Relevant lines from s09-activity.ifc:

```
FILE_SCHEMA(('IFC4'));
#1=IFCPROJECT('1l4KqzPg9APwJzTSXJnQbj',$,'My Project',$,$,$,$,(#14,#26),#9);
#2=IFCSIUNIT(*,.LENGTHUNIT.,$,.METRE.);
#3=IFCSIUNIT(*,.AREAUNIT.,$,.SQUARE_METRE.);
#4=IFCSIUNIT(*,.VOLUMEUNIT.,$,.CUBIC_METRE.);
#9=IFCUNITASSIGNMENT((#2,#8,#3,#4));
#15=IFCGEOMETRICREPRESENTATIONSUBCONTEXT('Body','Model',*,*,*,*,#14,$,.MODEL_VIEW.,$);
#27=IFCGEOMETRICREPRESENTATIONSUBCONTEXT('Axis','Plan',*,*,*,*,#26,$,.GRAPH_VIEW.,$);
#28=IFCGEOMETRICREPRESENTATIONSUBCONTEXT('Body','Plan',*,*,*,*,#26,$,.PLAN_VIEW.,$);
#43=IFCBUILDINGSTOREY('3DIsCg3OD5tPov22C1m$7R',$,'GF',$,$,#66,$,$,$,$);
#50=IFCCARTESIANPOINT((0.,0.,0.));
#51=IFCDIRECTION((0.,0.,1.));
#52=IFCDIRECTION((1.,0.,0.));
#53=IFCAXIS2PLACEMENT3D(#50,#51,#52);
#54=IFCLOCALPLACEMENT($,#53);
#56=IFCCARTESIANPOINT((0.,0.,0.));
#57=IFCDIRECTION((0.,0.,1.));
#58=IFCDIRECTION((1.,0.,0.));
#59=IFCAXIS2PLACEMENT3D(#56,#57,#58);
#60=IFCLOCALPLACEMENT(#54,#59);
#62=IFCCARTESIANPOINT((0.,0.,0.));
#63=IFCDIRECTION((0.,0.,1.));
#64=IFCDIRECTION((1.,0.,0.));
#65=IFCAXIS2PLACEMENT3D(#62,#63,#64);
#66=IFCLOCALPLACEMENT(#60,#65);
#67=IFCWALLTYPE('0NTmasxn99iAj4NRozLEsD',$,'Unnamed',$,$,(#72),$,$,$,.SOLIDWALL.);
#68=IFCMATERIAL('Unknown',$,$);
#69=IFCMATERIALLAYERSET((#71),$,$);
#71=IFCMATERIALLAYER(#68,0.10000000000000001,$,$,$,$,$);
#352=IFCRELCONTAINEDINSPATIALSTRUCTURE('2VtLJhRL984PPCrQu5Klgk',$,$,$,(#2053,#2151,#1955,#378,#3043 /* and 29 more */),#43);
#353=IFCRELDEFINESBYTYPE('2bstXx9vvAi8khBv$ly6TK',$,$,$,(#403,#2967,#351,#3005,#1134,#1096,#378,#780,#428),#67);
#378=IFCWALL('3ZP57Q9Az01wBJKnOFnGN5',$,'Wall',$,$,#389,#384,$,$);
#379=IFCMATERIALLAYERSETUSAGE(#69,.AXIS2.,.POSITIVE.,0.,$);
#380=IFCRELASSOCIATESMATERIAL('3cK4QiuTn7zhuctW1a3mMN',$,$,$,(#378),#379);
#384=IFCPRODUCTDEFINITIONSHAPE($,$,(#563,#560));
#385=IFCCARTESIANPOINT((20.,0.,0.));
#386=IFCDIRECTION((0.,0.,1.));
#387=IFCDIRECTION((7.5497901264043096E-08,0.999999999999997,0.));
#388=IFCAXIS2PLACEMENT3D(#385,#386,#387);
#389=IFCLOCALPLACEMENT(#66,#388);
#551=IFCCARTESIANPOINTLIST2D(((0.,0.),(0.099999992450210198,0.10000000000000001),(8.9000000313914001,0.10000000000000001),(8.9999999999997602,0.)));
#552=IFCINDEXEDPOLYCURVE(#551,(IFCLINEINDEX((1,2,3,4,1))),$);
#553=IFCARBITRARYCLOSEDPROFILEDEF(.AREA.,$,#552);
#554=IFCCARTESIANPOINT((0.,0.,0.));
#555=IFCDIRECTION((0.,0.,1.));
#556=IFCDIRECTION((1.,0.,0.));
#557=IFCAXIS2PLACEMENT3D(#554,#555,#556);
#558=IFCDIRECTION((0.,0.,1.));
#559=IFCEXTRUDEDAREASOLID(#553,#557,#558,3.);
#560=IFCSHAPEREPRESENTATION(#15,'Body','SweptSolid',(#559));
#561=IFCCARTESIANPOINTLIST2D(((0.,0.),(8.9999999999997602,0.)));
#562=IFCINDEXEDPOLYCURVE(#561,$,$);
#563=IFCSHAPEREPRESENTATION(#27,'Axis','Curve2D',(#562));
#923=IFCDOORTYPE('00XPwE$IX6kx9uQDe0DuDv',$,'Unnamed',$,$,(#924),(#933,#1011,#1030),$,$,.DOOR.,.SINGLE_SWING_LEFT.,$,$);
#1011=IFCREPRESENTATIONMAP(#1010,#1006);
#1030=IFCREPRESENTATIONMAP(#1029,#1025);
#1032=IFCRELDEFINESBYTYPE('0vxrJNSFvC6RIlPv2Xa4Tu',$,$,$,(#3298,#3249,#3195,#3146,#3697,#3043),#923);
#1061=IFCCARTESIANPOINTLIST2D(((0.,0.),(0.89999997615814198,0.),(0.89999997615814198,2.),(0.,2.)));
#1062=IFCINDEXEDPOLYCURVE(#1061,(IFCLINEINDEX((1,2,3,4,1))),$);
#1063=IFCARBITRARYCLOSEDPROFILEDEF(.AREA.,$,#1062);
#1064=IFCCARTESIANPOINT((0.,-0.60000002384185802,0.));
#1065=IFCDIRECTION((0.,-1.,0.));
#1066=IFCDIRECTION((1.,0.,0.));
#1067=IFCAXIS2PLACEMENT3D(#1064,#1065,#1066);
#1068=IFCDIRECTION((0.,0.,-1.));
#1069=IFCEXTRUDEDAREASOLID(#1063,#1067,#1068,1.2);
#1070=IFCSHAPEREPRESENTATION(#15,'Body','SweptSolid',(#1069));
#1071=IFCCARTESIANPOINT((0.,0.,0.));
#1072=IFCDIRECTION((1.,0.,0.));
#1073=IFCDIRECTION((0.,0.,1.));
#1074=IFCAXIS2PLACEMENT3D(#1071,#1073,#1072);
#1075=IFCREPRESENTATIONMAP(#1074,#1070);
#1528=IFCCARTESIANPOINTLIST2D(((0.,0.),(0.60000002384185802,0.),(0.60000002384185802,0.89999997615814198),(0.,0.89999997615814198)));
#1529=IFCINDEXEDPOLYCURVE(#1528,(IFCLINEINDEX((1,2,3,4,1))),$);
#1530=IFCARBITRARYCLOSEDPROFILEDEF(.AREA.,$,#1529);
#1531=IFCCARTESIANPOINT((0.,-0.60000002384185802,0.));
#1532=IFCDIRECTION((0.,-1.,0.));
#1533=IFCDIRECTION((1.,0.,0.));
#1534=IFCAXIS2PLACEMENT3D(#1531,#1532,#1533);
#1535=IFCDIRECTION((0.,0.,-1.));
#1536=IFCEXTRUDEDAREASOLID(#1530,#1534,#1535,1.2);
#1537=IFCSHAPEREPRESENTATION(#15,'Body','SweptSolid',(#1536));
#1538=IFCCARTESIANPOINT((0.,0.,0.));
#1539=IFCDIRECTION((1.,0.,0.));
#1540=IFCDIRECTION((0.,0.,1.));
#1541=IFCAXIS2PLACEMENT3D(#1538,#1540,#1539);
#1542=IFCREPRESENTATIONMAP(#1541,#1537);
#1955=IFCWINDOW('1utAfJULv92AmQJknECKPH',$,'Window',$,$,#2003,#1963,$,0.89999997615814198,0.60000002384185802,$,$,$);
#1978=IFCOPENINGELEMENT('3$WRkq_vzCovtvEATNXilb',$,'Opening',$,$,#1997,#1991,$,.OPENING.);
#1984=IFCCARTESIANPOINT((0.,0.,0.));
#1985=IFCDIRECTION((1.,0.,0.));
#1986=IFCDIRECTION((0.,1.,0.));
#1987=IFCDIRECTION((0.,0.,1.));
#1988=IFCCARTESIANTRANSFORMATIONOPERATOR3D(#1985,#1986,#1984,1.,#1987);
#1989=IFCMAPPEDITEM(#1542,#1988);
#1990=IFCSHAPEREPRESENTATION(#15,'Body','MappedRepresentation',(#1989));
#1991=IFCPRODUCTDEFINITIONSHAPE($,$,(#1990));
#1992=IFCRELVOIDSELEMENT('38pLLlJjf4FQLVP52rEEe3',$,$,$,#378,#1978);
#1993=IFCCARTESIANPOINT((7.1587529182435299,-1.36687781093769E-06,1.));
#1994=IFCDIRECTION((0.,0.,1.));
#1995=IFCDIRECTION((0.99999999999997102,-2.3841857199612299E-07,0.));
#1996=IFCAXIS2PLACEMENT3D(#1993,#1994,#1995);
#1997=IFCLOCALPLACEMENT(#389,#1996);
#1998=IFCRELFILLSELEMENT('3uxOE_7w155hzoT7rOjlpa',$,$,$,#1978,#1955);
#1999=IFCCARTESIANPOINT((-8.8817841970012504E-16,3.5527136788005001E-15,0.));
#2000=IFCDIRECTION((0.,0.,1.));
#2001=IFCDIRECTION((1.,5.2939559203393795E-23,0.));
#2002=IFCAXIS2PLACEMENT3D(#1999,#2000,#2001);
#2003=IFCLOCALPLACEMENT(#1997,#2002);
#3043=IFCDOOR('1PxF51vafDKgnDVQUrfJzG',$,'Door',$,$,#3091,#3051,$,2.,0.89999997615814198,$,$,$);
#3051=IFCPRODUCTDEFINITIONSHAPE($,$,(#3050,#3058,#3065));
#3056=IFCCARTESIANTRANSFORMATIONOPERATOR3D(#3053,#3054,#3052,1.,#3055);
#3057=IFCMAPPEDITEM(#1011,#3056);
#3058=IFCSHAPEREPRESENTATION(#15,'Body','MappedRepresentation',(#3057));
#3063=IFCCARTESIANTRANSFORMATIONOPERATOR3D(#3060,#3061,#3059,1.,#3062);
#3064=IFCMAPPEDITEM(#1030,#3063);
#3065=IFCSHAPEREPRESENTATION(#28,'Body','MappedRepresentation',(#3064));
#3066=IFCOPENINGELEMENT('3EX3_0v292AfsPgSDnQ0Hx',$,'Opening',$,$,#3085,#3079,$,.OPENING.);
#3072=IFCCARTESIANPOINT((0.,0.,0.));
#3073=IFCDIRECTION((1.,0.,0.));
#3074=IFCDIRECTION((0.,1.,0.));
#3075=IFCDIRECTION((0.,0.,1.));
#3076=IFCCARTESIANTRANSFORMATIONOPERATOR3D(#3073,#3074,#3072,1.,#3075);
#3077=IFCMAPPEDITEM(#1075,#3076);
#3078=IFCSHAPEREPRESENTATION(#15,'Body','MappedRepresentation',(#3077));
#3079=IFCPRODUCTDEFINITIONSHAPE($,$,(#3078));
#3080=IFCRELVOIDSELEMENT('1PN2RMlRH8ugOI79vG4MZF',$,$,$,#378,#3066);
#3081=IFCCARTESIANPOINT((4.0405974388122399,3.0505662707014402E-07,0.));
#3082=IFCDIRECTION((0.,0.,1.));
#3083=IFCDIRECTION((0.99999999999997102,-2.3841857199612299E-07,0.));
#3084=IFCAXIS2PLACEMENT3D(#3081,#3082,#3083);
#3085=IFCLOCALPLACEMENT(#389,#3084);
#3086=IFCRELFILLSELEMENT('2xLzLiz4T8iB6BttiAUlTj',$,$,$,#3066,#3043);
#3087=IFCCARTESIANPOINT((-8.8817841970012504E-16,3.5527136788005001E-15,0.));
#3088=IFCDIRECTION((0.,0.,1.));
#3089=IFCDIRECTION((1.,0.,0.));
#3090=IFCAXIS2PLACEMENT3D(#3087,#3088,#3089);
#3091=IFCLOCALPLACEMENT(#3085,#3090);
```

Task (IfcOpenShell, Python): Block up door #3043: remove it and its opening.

```python
import ifcopenshell
import ifcopenshell.api.feature
import ifcopenshell.api.root
import ifcopenshell.geom
import ifcopenshell.util.shape

model = ifcopenshell.open("s09-activity.ifc")
settings = ifcopenshell.geom.settings()


def volume(element):
    """Net volume in cubic metres, openings subtracted."""
    shape = ifcopenshell.geom.create_shape(settings, element)
    return ifcopenshell.util.shape.get_volume(shape.geometry)


door = model.by_id(3043)
opening = door.FillsVoids[0].RelatingOpeningElement
wall = opening.VoidsElements[0].RelatingBuildingElement
before = volume(wall)

ifcopenshell.api.root.remove_product(model, product=door)
ifcopenshell.api.feature.remove_feature(model, feature=opening)

after = volume(wall)

print(f"wall volume {before:.3f} -> {after:.3f} m3")

model.write("s09-activity_rev.ifc")
```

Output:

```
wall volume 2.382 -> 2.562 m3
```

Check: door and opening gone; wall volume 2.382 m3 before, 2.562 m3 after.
